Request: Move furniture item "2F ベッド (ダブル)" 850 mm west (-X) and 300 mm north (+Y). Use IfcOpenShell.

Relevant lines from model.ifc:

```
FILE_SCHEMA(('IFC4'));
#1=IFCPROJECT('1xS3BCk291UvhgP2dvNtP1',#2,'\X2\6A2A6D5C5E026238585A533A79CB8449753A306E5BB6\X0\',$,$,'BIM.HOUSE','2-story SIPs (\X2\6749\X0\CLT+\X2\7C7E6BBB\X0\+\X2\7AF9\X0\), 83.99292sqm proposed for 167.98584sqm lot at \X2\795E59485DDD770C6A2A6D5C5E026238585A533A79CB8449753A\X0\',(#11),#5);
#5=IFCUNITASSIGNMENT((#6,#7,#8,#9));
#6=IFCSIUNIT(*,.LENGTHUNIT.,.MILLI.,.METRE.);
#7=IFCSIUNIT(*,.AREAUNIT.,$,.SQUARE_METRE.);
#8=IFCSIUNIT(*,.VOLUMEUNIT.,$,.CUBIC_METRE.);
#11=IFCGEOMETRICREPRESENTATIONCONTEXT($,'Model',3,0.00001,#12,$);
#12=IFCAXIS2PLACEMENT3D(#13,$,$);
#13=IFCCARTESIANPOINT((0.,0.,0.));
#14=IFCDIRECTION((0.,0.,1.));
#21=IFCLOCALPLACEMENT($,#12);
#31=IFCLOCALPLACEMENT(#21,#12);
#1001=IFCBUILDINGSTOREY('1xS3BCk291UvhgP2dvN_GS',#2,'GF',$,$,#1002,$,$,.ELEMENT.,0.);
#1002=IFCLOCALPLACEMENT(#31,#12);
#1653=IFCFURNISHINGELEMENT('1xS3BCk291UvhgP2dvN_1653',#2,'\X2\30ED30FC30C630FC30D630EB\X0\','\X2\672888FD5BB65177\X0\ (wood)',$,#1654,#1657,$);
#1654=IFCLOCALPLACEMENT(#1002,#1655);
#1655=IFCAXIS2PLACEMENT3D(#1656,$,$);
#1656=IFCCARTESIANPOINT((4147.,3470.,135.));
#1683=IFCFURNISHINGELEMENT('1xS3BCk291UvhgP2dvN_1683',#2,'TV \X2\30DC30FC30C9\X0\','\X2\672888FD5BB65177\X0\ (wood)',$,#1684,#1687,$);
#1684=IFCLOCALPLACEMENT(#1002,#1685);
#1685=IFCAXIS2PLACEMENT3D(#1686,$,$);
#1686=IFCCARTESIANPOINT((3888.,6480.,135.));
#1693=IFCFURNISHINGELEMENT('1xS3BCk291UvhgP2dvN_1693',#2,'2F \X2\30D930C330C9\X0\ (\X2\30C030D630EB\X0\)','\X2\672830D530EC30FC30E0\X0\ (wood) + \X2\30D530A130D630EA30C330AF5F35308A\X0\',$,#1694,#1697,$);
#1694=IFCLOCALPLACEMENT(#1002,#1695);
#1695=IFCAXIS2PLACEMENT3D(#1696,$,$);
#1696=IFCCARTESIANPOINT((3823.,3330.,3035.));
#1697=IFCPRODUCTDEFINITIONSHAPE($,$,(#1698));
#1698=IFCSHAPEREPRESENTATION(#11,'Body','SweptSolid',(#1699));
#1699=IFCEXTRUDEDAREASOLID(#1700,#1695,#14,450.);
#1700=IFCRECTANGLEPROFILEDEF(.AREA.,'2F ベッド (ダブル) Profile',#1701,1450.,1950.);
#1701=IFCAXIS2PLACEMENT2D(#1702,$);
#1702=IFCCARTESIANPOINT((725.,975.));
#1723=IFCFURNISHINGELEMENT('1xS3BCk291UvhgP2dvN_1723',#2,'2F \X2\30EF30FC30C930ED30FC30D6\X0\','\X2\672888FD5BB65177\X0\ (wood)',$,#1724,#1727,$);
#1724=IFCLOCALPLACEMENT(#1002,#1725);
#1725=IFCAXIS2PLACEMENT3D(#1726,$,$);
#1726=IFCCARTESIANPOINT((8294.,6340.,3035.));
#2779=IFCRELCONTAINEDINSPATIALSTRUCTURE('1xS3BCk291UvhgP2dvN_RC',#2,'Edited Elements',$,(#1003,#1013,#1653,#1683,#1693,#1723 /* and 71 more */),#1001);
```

```python
import ifcopenshell
import ifcopenshell.api.geometry
import ifcopenshell.util.placement
import ifcopenshell.util.unit

model = ifcopenshell.open("model.ifc")
unit_scale = ifcopenshell.util.unit.calculate_unit_scale(model)

item = model.by_guid("1xS3BCk291UvhgP2dvN_1693")
matrix = ifcopenshell.util.placement.get_local_placement(item.ObjectPlacement)
matrix[0, 3] -= 0.85 / unit_scale
matrix[1, 3] += 0.3 / unit_scale
ifcopenshell.api.geometry.edit_object_placement(model, product=item, matrix=matrix, is_si=False)

print(ifcopenshell.util.placement.get_local_placement(item.ObjectPlacement).round(3) + 0.0)

model.write("model_rev.ifc")
```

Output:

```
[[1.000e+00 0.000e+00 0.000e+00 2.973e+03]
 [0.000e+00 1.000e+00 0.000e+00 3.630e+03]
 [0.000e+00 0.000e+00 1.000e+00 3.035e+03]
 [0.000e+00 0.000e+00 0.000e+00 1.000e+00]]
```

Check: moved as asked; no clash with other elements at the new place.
